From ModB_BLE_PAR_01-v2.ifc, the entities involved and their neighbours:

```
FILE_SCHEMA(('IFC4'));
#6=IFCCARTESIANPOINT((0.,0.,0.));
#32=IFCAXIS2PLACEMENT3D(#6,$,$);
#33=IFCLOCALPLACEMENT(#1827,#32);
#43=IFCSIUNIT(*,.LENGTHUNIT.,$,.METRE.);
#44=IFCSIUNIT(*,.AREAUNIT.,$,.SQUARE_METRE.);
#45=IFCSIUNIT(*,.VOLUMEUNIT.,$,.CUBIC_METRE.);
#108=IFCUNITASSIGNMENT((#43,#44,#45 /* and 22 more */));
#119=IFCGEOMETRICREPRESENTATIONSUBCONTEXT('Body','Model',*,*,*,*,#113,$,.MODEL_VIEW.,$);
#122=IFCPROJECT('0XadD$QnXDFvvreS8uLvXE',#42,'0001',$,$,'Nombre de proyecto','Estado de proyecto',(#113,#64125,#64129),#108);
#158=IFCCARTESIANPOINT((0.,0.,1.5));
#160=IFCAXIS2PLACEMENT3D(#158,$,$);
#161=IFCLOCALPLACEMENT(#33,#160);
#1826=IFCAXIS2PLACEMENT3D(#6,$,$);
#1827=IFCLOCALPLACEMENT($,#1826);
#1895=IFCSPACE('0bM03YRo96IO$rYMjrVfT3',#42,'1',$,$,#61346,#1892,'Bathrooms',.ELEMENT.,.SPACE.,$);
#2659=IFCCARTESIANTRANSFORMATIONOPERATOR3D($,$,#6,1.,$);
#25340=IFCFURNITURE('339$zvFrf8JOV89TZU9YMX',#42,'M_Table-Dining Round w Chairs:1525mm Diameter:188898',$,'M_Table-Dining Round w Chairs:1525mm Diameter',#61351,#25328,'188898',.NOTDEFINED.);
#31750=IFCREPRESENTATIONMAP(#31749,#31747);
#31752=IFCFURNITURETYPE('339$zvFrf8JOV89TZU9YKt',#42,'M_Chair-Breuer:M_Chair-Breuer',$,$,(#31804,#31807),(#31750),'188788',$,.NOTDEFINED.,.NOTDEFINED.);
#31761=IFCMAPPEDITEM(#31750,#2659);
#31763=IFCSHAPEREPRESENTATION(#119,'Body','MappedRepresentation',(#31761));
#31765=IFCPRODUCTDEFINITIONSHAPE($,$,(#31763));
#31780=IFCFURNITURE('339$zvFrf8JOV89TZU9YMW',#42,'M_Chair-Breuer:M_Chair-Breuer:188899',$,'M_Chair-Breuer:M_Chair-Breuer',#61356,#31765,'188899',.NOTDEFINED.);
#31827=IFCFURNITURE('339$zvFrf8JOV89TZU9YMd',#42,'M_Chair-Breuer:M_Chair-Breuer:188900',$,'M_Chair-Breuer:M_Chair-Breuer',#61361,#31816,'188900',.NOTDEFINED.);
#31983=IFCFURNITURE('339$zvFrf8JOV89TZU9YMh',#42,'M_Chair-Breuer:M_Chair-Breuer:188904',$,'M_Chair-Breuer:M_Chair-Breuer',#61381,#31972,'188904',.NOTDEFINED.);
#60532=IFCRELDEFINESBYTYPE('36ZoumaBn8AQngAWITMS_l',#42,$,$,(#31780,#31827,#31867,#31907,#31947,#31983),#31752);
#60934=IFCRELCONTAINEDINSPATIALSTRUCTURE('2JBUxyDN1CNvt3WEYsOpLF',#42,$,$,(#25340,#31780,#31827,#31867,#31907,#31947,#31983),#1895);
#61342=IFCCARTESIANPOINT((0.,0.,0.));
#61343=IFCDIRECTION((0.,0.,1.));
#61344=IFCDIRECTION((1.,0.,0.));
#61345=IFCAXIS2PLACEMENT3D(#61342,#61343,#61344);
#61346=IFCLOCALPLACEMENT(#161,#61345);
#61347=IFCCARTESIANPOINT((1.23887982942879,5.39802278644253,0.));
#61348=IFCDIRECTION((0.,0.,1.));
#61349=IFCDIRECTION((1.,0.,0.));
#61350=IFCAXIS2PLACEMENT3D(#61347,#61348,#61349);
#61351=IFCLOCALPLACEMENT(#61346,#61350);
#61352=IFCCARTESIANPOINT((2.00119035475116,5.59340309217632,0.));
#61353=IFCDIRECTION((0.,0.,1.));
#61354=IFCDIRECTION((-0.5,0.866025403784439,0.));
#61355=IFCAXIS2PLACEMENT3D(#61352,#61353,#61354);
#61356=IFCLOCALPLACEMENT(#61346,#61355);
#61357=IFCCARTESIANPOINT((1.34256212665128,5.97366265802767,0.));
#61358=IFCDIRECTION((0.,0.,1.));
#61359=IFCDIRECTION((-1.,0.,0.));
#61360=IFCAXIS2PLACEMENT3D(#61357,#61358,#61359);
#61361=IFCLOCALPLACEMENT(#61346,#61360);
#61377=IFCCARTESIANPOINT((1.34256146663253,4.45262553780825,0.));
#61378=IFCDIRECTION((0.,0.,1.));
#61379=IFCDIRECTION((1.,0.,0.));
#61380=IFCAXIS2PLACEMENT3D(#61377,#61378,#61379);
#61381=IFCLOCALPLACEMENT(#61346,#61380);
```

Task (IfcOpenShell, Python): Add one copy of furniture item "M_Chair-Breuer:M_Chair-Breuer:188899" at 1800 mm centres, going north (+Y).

```python
import numpy as np
import ifcopenshell
import ifcopenshell.api.geometry
import ifcopenshell.api.root
import ifcopenshell.util.element
import ifcopenshell.util.placement
import ifcopenshell.util.unit

model = ifcopenshell.open("ModB_BLE_PAR_01-v2.ifc")
unit_scale = ifcopenshell.util.unit.calculate_unit_scale(model)


def reuse_history(source, copy):
    """copy_class also copies each property set's owner history, people and application; keep the originals."""
    for rel in copy.IsDefinedBy:
        if rel.is_a("IfcRelDefinesByProperties") and (history := rel.RelatingPropertyDefinition.OwnerHistory):
            rel.RelatingPropertyDefinition.OwnerHistory = source.OwnerHistory
            ifcopenshell.util.element.remove_deep2(model, history)


source = model.by_id(31780)
base = ifcopenshell.util.placement.get_local_placement(source.ObjectPlacement)
step = np.array([0.0, 1.0, 0.0]) * 1.8 / unit_scale

for i in range(1, 2):
    copy = ifcopenshell.api.root.copy_class(model, product=source)
    copy.Representation = ifcopenshell.util.element.copy_deep(
        model, source.Representation, exclude=["IfcGeometricRepresentationContext", "IfcRepresentationMap"]
    )
    copy.Name = "M_Chair-Breuer:M_Chair-Breuer"
    copy.Tag = None
    reuse_history(source, copy)
    matrix = base.copy()
    matrix[:3, 3] += i * step
    print("added at", matrix[:3, 3].round(3) + 0.0)
    ifcopenshell.api.geometry.edit_object_placement(model, product=copy, matrix=matrix, is_si=False)

model.write("ModB_BLE_PAR_01-v2_updated.ifc")
```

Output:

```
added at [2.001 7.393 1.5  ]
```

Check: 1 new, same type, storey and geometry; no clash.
